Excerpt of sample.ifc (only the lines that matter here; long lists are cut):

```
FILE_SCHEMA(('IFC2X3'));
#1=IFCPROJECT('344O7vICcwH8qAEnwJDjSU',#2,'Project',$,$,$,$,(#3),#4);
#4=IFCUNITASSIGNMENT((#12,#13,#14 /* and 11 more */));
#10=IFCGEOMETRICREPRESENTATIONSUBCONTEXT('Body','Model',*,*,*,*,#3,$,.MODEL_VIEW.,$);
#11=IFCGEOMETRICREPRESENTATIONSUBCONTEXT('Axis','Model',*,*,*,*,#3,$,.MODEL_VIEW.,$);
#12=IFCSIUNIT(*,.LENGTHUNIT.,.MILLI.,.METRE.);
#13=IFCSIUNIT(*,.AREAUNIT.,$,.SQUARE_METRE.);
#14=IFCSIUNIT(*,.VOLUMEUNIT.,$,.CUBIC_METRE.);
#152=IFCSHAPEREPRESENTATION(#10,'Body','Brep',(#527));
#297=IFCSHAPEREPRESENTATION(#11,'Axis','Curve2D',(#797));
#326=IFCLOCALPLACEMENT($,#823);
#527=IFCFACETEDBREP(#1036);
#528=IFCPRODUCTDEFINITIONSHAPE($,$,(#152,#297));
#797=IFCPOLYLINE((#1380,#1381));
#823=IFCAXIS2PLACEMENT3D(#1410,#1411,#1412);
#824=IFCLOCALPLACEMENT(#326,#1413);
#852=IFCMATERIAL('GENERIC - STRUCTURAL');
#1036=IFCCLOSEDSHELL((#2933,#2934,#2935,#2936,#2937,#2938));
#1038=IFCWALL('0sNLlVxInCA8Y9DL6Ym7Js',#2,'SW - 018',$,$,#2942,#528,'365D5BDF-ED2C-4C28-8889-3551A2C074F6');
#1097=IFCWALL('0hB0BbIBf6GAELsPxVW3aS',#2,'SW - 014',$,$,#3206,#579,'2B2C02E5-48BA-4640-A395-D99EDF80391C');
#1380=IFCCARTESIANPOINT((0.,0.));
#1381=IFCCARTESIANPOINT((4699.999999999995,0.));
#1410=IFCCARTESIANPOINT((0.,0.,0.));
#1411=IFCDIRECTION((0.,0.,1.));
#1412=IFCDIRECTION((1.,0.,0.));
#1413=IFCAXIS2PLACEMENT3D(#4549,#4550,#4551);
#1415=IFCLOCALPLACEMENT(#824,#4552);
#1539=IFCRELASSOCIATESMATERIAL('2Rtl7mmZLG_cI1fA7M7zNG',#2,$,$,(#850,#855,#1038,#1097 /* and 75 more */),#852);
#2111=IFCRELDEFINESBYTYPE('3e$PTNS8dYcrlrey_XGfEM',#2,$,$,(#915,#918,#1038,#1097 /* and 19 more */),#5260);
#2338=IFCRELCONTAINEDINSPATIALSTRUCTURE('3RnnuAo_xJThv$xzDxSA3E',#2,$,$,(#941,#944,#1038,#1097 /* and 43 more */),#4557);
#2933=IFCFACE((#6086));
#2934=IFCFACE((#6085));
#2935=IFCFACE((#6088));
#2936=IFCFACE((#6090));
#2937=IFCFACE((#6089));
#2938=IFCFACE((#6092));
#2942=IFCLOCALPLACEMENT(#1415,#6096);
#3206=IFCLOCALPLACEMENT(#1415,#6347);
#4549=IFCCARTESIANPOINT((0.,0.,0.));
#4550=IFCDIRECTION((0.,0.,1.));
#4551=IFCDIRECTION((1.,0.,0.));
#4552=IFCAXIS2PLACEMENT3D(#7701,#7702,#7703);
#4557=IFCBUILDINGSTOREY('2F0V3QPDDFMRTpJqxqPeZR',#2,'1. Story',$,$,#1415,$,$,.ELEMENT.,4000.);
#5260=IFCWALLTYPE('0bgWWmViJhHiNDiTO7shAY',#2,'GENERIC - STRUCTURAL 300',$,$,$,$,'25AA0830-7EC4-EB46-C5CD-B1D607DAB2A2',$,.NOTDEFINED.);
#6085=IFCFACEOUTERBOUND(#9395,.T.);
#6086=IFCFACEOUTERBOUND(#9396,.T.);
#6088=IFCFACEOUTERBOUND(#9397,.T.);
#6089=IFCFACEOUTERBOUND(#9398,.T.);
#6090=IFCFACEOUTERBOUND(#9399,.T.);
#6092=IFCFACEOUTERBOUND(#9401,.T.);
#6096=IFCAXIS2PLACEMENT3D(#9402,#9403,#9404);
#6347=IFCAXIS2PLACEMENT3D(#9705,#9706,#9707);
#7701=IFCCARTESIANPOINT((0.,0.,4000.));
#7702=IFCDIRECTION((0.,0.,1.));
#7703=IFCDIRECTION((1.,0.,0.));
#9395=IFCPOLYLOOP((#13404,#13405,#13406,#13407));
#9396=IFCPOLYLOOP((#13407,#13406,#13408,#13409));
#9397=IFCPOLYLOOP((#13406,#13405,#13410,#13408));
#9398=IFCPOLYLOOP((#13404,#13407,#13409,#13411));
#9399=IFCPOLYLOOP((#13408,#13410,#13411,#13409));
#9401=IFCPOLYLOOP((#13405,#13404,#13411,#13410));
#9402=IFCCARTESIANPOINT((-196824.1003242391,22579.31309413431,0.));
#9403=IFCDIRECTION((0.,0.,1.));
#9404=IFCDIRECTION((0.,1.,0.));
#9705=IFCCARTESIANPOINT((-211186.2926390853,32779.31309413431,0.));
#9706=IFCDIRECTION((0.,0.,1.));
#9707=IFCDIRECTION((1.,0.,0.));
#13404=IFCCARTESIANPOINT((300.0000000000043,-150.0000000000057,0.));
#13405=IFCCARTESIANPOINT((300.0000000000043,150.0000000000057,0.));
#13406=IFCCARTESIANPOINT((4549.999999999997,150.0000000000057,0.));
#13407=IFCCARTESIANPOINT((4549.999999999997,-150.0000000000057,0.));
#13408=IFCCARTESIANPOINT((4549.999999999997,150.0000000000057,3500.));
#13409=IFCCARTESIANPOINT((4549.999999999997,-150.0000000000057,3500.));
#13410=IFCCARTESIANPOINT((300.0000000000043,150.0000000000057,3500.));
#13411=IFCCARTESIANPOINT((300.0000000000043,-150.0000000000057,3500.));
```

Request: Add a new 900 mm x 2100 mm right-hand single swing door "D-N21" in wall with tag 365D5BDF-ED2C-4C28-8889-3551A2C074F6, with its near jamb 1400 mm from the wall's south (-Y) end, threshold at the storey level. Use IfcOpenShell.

```python
import numpy as np
import ifcopenshell
import ifcopenshell.api.feature
import ifcopenshell.api.geometry
import ifcopenshell.api.root
import ifcopenshell.api.spatial
import ifcopenshell.api.type
import ifcopenshell.geom
import ifcopenshell.util.element
import ifcopenshell.util.placement
import ifcopenshell.util.representation
import ifcopenshell.util.shape
import ifcopenshell.util.unit

model = ifcopenshell.open("sample.ifc")
unit_scale = ifcopenshell.util.unit.calculate_unit_scale(model)
settings = ifcopenshell.geom.settings()


def volume(element):
    """Net volume in cubic metres, openings subtracted."""
    shape = ifcopenshell.geom.create_shape(settings, element)
    return ifcopenshell.util.shape.get_volume(shape.geometry)


wall = model.by_id(1038)
storey = ifcopenshell.util.element.get_container(wall, ifc_class="IfcBuildingStorey")
context = ifcopenshell.util.representation.get_context(model, "Model", "Body", "MODEL_VIEW")
before = volume(wall)

width, height, from_end, sill = 0.9, 2.1, 1.4, 0.0  # metres

# The wall runs along its own X axis, and the end named is its -X end.
wall_shape = ifcopenshell.geom.create_shape(settings, wall)
x, y, z = ifcopenshell.util.shape.get_vertices(wall_shape.geometry).T
start = x.min() + from_end
face, thickness = float(y.min()), float(y.max() - y.min())
wall_matrix = ifcopenshell.util.placement.get_local_placement(wall.ObjectPlacement)
level = ifcopenshell.util.placement.get_local_placement(storey.ObjectPlacement)[2, 3]


def in_wall(x, y):
    """Placement at x, y metres in the wall's axes, at sill height."""
    matrix = wall_matrix.copy()
    matrix[:, 3] = wall_matrix @ np.array([x / unit_scale, y / unit_scale, 0.0, 1.0])
    matrix[2, 3] = level + sill / unit_scale
    return matrix


# Opening: a box that overshoots both wall faces by 50 mm.
opening = ifcopenshell.api.root.create_entity(model, ifc_class="IfcOpeningElement")
box = ifcopenshell.api.geometry.add_wall_representation(
    model, context=context, length=width, height=height, thickness=thickness + 0.1
)
ifcopenshell.api.geometry.assign_representation(model, product=opening, representation=box)
ifcopenshell.api.geometry.edit_object_placement(model, product=opening, matrix=in_wall(start, face - 0.05), is_si=False)
ifcopenshell.api.feature.add_feature(model, feature=opening, element=wall)

door = ifcopenshell.api.root.create_entity(model, ifc_class="IfcDoor", name="D-N21")
door.OverallWidth, door.OverallHeight = width / unit_scale, height / unit_scale
body = ifcopenshell.api.geometry.add_door_representation(
    model,
    context=context,
    overall_width=door.OverallWidth,
    overall_height=door.OverallHeight,
    operation_type="SINGLE_SWING_RIGHT",
    lining_properties={"LiningDepth": thickness / unit_scale, "ThresholdDepth": thickness / unit_scale},
)
ifcopenshell.api.geometry.assign_representation(model, product=door, representation=body)
ifcopenshell.api.spatial.assign_container(model, products=[door], relating_structure=storey)
fills = ifcopenshell.api.feature.add_filling(model, opening=opening, element=door)
fills.OwnerHistory = door.OwnerHistory  # required in IFC2X3

# IFC2X3 keeps the operation on the door style.
style = ifcopenshell.api.root.create_entity(model, ifc_class="IfcDoorStyle", name="D-N21")
style.OperationType, style.ConstructionType = "SINGLE_SWING_RIGHT", "NOTDEFINED"
style.ParameterTakesPrecedence = style.Sizeable = False
ifcopenshell.api.type.assign_type(model, related_objects=[door], relating_type=style)

# The lining spans the wall, so the door starts at the wall face.
ifcopenshell.api.geometry.edit_object_placement(model, product=door, matrix=in_wall(start, face), is_si=False)

after = volume(wall)

print(f"wall volume {before:.3f} -> {after:.3f} m3")

model.write("sample_v2.ifc")
```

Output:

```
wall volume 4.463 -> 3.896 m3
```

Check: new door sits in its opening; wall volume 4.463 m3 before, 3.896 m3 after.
